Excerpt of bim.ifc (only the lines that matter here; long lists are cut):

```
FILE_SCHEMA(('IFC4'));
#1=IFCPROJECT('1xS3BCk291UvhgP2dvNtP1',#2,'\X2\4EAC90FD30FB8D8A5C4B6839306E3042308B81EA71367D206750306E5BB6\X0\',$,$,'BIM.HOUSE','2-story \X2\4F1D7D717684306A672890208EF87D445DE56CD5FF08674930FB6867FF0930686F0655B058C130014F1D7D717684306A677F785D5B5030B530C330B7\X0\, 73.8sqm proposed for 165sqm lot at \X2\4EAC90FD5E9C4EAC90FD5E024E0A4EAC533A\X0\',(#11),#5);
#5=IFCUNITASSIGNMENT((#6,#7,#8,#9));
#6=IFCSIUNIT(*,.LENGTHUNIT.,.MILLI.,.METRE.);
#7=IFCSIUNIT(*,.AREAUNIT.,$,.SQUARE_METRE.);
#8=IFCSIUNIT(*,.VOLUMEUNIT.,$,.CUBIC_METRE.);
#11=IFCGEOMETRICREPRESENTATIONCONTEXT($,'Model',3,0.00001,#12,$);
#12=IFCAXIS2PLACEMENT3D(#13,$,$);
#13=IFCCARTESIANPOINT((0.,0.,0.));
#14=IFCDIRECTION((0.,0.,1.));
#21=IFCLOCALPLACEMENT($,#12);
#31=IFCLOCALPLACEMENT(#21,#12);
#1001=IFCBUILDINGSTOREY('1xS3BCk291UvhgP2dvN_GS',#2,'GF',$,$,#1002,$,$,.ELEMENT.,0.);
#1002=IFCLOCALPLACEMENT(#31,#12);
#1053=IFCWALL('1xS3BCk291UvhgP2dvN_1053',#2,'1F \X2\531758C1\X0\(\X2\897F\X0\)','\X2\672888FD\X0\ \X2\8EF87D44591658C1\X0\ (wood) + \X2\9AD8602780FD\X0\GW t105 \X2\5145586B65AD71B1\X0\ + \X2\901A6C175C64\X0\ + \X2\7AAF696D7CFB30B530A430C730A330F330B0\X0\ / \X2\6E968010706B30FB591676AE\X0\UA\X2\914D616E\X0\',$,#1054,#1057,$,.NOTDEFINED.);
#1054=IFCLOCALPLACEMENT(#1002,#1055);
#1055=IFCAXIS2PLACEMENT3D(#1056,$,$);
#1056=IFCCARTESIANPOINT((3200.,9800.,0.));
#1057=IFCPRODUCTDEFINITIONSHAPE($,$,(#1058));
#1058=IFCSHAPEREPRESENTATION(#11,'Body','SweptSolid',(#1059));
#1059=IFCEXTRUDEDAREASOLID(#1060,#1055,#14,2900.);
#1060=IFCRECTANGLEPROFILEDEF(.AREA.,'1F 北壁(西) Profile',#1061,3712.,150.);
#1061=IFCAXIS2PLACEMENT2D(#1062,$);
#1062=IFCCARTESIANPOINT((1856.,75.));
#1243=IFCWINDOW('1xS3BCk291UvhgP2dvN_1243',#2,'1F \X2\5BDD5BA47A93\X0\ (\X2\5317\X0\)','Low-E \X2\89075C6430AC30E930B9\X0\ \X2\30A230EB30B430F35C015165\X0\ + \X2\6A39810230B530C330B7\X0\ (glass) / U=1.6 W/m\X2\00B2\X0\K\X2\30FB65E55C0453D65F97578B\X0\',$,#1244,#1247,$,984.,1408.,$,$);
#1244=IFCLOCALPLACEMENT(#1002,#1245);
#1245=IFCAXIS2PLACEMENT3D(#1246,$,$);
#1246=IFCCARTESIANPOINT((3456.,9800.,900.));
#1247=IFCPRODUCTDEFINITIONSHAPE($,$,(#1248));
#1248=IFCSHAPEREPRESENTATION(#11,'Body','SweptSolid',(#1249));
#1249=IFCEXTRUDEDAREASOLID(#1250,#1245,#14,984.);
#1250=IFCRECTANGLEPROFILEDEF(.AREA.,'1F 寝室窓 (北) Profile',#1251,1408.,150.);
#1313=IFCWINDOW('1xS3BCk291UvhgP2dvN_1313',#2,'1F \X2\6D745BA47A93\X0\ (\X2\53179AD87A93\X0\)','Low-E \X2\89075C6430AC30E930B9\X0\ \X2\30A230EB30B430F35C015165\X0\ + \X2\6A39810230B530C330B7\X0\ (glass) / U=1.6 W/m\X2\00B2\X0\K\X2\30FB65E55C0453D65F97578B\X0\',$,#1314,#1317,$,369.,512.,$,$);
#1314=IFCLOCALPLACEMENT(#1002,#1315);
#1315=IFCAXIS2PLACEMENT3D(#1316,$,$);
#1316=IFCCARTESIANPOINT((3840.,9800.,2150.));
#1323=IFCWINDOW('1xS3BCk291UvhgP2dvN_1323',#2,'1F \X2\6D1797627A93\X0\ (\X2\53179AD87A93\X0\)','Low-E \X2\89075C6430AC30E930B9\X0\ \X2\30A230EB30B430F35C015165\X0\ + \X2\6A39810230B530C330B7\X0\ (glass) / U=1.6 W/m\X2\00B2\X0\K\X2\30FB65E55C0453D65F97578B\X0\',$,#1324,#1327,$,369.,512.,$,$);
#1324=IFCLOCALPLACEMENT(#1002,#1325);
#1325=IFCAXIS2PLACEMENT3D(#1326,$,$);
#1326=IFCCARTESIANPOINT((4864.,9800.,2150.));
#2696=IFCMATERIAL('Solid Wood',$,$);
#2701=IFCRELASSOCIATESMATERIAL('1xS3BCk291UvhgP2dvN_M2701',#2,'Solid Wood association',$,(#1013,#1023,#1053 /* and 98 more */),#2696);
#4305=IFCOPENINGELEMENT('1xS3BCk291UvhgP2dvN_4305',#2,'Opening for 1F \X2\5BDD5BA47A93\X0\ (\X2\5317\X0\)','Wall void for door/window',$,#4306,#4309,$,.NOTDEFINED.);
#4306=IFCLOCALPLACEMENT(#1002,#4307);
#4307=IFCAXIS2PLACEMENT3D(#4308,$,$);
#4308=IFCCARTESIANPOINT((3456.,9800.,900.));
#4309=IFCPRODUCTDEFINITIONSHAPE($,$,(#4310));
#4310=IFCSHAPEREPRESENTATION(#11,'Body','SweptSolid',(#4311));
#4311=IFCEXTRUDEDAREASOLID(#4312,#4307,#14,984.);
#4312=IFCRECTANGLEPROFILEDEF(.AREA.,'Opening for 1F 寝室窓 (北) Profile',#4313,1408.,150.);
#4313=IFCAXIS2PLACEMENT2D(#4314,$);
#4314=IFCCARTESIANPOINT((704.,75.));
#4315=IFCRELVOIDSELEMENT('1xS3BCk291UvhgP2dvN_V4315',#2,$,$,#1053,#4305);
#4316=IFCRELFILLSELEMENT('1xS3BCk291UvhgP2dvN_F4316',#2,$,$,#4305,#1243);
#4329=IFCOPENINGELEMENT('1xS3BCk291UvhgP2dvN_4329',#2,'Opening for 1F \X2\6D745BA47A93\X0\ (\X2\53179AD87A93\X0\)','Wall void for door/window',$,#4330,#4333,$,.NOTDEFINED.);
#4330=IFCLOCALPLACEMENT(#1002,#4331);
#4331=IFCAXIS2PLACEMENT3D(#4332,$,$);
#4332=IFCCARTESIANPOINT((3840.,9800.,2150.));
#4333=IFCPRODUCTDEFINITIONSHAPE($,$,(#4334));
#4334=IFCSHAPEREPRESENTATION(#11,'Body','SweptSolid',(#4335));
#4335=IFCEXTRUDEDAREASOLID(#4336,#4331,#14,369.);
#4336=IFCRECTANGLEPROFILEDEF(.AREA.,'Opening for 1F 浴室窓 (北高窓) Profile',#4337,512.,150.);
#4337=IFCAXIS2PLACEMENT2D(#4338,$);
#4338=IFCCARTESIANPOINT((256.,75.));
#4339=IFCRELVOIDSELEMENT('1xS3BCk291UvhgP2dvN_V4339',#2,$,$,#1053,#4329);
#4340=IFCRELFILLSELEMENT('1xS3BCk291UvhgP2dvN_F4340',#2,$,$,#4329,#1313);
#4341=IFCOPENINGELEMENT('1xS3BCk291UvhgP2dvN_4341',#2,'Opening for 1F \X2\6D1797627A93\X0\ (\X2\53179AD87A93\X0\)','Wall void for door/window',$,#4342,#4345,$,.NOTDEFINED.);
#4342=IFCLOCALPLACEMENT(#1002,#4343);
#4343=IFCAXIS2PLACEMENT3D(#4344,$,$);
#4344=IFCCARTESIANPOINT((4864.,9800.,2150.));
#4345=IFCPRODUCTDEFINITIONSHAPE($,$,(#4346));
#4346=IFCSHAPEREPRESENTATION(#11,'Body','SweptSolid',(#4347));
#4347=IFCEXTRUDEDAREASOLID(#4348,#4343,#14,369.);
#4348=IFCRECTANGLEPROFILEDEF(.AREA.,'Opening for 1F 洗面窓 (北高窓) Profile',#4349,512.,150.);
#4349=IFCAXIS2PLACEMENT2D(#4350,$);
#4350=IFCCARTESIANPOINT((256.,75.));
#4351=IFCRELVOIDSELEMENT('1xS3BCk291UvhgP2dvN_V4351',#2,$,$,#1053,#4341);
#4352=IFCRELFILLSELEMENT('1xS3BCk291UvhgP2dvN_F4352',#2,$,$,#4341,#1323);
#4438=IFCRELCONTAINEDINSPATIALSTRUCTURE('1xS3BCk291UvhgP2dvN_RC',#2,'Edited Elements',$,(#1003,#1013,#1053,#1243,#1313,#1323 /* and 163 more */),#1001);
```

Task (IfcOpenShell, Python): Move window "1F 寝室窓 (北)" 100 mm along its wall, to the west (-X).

```python
import ifcopenshell
import ifcopenshell.api.geometry
import ifcopenshell.util.placement

model = ifcopenshell.open("bim.ifc")

window = model.by_guid("1xS3BCk291UvhgP2dvN_1243")
opening = window.FillsVoids[0].RelatingOpeningElement
wall = opening.VoidsElements[0].RelatingBuildingElement

wall_matrix = ifcopenshell.util.placement.get_local_placement(wall.ObjectPlacement)
shift = wall_matrix[:3, 0] * -100.0
before = ifcopenshell.util.placement.get_local_placement(window.ObjectPlacement)[:3, 3].copy()

# The window is not placed relative to its opening, so move both.
for product in (opening, window):
    matrix = ifcopenshell.util.placement.get_local_placement(product.ObjectPlacement)
    matrix[:3, 3] += shift
    ifcopenshell.api.geometry.edit_object_placement(model, product=product, matrix=matrix, is_si=False)

after = ifcopenshell.util.placement.get_local_placement(window.ObjectPlacement)[:3, 3]
print("window moved by", (after - before).round(3) + 0.0)

model.write("bim_rev.ifc")
```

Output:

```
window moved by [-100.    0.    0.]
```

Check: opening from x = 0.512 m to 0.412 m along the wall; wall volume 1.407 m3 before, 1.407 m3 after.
